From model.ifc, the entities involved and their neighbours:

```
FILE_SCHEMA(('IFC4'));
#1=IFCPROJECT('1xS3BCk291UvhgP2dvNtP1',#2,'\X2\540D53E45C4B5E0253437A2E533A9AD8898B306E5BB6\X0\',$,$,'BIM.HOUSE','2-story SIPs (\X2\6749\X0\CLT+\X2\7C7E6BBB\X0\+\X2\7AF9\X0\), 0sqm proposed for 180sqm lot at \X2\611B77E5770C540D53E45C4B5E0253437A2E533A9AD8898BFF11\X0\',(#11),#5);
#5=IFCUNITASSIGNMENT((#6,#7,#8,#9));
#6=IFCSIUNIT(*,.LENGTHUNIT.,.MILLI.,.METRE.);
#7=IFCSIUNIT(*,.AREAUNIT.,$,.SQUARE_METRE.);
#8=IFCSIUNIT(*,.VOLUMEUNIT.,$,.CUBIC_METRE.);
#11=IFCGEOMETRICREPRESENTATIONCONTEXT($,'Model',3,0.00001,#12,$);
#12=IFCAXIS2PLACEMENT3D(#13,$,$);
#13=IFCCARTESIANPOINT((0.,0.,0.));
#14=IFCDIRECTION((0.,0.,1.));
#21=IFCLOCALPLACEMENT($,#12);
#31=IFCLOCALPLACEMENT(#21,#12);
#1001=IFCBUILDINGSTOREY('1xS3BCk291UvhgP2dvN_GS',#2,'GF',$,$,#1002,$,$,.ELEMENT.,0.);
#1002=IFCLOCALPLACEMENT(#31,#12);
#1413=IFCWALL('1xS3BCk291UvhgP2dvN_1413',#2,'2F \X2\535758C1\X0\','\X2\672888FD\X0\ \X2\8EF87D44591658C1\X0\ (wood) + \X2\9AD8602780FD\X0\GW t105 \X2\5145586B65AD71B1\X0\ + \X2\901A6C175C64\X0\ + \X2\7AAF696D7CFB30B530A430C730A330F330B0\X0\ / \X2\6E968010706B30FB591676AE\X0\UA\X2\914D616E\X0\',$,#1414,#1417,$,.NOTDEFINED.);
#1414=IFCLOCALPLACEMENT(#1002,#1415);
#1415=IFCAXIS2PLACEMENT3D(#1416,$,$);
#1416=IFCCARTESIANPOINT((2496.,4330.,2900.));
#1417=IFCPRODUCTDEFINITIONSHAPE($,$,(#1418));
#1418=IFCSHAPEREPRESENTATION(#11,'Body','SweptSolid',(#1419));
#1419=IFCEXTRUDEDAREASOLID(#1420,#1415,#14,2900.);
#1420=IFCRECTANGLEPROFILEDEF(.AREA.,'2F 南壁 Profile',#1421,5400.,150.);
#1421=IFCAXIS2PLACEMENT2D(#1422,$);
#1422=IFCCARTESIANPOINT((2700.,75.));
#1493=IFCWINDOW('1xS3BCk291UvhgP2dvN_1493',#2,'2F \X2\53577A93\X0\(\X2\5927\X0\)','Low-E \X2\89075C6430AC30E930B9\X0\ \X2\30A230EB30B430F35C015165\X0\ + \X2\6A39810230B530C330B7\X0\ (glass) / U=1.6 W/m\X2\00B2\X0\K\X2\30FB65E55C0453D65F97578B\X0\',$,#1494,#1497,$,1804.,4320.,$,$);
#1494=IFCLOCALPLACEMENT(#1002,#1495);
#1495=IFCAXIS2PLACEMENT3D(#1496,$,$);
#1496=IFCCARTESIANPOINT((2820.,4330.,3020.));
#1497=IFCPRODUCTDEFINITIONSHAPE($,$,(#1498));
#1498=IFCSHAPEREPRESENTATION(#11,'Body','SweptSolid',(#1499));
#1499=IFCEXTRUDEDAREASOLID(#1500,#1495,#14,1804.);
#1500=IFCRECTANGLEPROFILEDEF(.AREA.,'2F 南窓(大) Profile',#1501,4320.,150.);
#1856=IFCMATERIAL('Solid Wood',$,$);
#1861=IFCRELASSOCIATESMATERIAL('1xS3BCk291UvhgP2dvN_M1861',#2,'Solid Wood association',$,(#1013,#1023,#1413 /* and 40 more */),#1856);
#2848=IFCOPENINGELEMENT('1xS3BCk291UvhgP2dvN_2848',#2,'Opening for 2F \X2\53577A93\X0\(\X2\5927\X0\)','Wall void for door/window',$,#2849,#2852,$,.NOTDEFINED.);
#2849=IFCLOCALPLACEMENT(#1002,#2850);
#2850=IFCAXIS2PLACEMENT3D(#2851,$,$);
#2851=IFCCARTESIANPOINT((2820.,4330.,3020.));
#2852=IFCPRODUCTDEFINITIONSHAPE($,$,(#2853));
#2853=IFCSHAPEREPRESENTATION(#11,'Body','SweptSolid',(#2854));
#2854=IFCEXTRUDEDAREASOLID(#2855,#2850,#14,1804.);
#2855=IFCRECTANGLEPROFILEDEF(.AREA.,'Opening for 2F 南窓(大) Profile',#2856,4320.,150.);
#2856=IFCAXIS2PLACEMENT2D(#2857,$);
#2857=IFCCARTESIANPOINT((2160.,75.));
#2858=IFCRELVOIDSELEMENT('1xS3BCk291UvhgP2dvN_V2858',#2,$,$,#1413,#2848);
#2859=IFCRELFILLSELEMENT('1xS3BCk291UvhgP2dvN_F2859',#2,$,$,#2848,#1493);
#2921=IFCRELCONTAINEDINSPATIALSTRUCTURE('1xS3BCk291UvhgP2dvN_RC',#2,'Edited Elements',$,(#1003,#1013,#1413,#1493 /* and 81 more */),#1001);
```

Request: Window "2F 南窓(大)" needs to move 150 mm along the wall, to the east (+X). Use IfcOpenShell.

```python
import ifcopenshell
import ifcopenshell.api.geometry
import ifcopenshell.util.placement
import ifcopenshell.util.unit

model = ifcopenshell.open("model.ifc")
unit_scale = ifcopenshell.util.unit.calculate_unit_scale(model)

window = model.by_id(1493)
opening = window.FillsVoids[0].RelatingOpeningElement
wall = opening.VoidsElements[0].RelatingBuildingElement

wall_matrix = ifcopenshell.util.placement.get_local_placement(wall.ObjectPlacement)
shift = wall_matrix[:3, 0] * 0.15 / unit_scale
before = ifcopenshell.util.placement.get_local_placement(window.ObjectPlacement)[:3, 3].copy()

# The window is not placed relative to its opening, so move both.
for product in (opening, window):
    matrix = ifcopenshell.util.placement.get_local_placement(product.ObjectPlacement)
    matrix[:3, 3] += shift
    ifcopenshell.api.geometry.edit_object_placement(model, product=product, matrix=matrix, is_si=False)

after = ifcopenshell.util.placement.get_local_placement(window.ObjectPlacement)[:3, 3]
print("window moved by", (after - before).round(3) + 0.0)

model.write("model_v2.ifc")
```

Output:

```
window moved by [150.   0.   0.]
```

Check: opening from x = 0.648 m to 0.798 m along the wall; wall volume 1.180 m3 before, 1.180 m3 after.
